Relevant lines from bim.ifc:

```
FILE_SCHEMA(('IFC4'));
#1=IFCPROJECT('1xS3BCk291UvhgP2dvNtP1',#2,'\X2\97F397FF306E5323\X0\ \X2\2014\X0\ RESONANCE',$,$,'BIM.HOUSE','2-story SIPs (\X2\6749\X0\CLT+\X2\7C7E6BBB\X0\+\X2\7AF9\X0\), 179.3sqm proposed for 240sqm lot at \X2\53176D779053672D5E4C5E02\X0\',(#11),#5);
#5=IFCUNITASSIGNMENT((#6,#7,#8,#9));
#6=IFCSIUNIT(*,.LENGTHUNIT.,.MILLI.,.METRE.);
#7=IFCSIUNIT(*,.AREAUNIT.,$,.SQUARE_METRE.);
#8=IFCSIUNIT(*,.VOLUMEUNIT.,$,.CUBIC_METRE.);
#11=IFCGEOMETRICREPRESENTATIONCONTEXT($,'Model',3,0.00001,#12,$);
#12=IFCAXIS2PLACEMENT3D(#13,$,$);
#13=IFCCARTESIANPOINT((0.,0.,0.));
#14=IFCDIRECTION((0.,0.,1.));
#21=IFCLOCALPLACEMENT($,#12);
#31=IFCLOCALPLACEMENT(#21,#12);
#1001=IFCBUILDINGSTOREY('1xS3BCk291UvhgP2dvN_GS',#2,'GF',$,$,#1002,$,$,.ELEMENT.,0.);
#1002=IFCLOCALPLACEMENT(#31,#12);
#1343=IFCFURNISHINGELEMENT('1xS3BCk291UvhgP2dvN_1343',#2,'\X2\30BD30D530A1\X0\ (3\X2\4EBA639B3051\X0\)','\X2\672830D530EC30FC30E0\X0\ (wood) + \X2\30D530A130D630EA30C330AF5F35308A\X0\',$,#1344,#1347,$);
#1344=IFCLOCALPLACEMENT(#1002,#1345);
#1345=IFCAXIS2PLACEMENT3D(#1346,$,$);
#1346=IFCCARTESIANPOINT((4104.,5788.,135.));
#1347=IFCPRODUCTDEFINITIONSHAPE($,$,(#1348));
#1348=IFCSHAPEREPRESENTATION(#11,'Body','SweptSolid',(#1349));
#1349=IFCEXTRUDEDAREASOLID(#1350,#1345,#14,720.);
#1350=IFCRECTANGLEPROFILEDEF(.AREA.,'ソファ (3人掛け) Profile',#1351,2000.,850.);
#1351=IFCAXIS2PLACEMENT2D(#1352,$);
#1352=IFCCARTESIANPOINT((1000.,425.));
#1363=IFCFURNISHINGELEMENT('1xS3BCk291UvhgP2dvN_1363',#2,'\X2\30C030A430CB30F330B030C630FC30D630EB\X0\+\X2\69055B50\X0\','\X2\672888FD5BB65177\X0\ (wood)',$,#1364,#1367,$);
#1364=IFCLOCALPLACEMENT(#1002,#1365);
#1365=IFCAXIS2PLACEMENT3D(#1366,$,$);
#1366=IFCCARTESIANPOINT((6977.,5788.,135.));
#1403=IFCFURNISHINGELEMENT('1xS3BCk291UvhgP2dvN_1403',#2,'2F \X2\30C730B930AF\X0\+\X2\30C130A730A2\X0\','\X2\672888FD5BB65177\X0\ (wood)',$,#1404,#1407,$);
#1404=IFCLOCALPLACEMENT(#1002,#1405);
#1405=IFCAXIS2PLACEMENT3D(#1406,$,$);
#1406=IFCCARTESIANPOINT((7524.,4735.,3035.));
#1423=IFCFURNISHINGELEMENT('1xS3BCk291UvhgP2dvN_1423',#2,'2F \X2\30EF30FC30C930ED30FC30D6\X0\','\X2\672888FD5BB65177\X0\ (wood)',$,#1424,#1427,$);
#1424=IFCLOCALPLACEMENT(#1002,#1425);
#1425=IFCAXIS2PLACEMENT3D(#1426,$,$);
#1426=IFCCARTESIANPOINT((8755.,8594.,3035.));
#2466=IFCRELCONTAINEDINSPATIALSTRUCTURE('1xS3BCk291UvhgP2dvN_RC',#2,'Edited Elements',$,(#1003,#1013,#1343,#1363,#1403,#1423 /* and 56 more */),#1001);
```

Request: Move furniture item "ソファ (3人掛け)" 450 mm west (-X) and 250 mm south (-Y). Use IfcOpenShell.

```python
import ifcopenshell
import ifcopenshell.api.geometry
import ifcopenshell.util.placement

model = ifcopenshell.open("bim.ifc")

item = model.by_guid("1xS3BCk291UvhgP2dvN_1343")
matrix = ifcopenshell.util.placement.get_local_placement(item.ObjectPlacement)
matrix[0, 3] -= 450.0
matrix[1, 3] -= 250.0
ifcopenshell.api.geometry.edit_object_placement(model, product=item, matrix=matrix, is_si=False)

print(ifcopenshell.util.placement.get_local_placement(item.ObjectPlacement).round(3) + 0.0)

model.write("bim_v2.ifc")
```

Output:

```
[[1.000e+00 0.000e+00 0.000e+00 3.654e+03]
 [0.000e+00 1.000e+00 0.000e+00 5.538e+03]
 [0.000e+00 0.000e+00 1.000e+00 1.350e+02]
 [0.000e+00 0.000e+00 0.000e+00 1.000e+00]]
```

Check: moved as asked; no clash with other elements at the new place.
